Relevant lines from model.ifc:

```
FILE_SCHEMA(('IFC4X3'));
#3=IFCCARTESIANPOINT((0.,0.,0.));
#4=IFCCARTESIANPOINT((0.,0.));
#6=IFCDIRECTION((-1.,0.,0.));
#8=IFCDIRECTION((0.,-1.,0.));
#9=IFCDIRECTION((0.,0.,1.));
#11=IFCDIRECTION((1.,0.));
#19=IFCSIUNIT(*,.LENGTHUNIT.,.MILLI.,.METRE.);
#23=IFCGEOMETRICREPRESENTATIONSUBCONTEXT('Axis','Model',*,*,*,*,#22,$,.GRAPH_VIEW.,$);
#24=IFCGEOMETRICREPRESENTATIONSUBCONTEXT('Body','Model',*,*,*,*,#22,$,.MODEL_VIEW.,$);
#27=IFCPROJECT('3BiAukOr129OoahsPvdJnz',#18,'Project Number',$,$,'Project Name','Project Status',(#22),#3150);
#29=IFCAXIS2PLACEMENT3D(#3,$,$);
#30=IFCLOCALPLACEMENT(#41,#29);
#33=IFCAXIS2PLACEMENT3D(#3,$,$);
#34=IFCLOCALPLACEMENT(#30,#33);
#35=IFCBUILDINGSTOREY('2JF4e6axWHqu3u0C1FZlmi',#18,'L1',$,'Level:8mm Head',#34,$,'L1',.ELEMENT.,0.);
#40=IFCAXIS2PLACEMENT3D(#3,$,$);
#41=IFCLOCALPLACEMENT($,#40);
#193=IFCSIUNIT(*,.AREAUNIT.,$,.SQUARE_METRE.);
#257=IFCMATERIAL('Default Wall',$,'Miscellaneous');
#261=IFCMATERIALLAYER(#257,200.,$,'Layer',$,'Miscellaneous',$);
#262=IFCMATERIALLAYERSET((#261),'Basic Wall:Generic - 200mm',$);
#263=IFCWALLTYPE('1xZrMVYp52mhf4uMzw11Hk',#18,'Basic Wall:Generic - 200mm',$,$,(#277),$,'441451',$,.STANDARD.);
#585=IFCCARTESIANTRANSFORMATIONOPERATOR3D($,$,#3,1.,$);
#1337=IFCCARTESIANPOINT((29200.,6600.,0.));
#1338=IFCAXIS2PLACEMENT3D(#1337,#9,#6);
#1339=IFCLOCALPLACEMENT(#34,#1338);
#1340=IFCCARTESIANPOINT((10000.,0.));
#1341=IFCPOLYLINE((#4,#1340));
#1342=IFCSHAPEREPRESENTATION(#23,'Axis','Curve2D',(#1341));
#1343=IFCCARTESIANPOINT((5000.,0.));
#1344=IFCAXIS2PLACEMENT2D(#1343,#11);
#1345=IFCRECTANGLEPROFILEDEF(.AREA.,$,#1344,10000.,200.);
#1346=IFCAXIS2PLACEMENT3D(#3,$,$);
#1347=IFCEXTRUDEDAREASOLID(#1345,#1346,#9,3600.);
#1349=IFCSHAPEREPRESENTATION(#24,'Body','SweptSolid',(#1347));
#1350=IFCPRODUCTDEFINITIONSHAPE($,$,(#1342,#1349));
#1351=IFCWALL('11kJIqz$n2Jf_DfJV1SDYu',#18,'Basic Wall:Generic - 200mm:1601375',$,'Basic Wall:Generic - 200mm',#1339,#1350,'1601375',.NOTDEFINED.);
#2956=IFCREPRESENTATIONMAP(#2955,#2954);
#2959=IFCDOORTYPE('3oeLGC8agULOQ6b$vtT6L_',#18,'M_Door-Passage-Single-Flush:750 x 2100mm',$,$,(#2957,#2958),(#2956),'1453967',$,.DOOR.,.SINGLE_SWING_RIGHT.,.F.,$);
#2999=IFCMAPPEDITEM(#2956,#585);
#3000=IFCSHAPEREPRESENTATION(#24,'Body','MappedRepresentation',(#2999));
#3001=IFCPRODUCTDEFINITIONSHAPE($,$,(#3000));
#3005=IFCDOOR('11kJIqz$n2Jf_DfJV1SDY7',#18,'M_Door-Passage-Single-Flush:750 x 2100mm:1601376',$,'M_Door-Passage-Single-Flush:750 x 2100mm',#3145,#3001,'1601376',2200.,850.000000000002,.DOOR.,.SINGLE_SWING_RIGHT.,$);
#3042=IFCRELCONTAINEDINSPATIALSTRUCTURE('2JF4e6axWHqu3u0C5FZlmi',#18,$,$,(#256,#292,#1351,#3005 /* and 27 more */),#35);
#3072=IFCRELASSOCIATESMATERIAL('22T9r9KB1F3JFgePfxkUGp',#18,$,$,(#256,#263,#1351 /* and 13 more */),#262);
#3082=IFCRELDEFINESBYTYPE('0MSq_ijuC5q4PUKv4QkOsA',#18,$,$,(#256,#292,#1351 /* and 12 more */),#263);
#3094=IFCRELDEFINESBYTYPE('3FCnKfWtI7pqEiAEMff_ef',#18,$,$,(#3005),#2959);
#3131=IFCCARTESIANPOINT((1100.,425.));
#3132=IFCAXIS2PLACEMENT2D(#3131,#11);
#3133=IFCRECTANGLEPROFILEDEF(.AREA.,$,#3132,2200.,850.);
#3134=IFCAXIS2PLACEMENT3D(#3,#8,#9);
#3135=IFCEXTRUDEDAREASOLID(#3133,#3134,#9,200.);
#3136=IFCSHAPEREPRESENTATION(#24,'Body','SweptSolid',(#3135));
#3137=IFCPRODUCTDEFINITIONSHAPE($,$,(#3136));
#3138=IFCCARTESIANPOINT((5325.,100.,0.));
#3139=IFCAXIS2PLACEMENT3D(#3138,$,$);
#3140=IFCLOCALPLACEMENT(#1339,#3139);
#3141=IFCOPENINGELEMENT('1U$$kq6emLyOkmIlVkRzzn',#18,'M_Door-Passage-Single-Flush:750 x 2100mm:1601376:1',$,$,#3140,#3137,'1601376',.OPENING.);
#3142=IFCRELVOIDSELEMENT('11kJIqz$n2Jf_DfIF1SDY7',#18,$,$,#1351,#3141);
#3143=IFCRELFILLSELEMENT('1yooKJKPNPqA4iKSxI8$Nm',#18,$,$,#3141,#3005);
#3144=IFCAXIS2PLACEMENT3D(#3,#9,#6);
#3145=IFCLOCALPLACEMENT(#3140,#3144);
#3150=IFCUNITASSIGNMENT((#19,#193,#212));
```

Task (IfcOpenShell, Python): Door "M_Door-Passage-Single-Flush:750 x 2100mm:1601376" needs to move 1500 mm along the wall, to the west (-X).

```python
import ifcopenshell
import ifcopenshell.api.geometry
import ifcopenshell.util.placement

model = ifcopenshell.open("model.ifc")

door = model.by_id(3005)
opening = door.FillsVoids[0].RelatingOpeningElement
wall = opening.VoidsElements[0].RelatingBuildingElement

wall_matrix = ifcopenshell.util.placement.get_local_placement(wall.ObjectPlacement)
shift = wall_matrix[:3, 0] * 1500.0
before = ifcopenshell.util.placement.get_local_placement(door.ObjectPlacement)[:3, 3].copy()

# The door is placed relative to its opening, so it follows when the opening moves.
matrix = ifcopenshell.util.placement.get_local_placement(opening.ObjectPlacement)
matrix[:3, 3] += shift
ifcopenshell.api.geometry.edit_object_placement(
    model, product=opening, matrix=matrix, is_si=False, should_transform_children=True
)

after = ifcopenshell.util.placement.get_local_placement(door.ObjectPlacement)[:3, 3]
print("door moved by", (after - before).round(3) + 0.0)

model.write("model_edited.ifc")
```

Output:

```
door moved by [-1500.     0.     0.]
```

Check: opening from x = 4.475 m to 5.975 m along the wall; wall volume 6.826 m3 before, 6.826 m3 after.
